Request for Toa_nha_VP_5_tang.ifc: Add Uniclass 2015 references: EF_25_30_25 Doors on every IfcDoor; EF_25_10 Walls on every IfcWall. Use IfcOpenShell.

First a look at what the model holds.

```python
import ifcopenshell

model = ifcopenshell.open("Toa_nha_VP_5_tang.ifc")
print(model.schema)
print("classifications:", [c.Name for c in model.by_type("IfcClassification")])
for ifc_class in ("IfcDoor", "IfcRoof", "IfcStair", "IfcWall", "IfcWindow"):
    print(ifc_class, len(model.by_type(ifc_class)))
```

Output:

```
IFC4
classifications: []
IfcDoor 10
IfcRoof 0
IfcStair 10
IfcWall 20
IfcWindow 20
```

```python
import ifcopenshell
import ifcopenshell.api.classification

model = ifcopenshell.open("Toa_nha_VP_5_tang.ifc")

system = ifcopenshell.api.classification.add_classification(model, classification="Uniclass 2015")

codes = {
    "IfcDoor": ("EF_25_30_25", "Doors"),
    "IfcWall": ("EF_25_10", "Walls"),
}
for ifc_class, (code, name) in codes.items():
    products = model.by_type(ifc_class)
    ifcopenshell.api.classification.add_reference(
        model, products=products, classification=system, identification=code, name=name
    )
    print(code, len(products))

model.write("Toa_nha_VP_5_tang-out.ifc")
```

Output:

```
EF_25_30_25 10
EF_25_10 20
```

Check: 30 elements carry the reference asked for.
